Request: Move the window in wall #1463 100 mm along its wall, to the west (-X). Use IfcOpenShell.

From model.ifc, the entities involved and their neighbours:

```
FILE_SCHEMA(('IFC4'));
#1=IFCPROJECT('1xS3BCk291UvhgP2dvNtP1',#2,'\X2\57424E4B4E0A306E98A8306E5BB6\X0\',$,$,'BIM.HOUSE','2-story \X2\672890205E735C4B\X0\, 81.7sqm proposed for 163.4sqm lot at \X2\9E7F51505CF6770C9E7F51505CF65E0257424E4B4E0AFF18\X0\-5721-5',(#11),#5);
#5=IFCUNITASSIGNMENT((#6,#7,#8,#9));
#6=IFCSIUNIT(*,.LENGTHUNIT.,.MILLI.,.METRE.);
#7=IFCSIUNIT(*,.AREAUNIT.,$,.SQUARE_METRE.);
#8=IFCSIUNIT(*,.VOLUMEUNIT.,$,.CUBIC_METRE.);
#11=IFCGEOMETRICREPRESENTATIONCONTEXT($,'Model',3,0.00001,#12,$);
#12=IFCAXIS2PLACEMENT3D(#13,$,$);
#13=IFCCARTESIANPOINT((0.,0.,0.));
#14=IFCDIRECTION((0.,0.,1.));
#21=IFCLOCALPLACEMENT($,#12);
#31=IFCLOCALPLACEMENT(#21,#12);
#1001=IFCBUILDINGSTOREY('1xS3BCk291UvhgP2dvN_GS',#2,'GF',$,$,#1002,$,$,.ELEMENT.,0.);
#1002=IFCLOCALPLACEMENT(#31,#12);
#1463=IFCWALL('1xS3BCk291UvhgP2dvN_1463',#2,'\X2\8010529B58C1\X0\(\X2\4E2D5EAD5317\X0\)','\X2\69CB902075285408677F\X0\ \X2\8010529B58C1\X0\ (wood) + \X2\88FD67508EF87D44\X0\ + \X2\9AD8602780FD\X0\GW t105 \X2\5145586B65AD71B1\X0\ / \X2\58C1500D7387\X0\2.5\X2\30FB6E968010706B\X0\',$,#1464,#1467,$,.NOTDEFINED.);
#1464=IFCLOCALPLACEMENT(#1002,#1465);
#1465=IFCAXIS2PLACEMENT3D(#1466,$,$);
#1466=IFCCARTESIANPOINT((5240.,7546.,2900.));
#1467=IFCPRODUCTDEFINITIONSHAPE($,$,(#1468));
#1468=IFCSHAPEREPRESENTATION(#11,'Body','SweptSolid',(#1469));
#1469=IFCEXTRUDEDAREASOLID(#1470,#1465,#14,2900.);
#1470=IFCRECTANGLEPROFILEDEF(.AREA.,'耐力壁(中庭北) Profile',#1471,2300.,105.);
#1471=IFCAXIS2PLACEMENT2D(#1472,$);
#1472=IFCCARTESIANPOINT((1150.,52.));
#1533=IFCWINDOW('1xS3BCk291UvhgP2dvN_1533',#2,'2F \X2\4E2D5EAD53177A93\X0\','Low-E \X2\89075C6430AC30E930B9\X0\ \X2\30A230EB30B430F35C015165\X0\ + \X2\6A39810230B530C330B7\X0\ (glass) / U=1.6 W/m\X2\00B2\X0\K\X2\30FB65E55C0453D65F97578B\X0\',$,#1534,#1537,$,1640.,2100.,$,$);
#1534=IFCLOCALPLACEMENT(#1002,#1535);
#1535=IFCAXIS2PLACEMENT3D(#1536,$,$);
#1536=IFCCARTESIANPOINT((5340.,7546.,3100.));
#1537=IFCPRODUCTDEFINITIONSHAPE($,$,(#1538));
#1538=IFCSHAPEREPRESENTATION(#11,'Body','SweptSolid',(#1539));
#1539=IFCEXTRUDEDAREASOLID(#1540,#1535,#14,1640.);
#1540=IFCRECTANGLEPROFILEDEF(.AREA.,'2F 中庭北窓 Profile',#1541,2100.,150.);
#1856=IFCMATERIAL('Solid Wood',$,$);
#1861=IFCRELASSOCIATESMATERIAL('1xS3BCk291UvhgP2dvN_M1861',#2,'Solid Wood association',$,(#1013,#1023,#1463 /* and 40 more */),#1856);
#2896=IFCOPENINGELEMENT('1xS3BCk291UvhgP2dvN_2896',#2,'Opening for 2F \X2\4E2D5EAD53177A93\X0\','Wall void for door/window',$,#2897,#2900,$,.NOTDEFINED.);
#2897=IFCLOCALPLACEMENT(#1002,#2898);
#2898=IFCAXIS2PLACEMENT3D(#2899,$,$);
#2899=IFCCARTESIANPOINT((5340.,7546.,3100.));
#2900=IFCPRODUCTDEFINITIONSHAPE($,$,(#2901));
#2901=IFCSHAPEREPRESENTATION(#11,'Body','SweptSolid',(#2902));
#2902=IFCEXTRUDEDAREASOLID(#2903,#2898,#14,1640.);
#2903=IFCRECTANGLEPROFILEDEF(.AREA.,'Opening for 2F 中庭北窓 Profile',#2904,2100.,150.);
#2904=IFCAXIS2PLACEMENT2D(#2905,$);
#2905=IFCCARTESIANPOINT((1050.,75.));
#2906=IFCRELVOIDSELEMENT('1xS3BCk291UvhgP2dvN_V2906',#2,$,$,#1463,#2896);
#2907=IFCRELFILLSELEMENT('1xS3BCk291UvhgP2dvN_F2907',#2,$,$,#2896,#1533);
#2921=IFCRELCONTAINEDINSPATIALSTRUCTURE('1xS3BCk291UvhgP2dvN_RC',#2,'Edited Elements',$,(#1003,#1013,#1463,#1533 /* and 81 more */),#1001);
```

```python
import ifcopenshell
import ifcopenshell.api.geometry
import ifcopenshell.util.placement
import ifcopenshell.util.unit

model = ifcopenshell.open("model.ifc")
unit_scale = ifcopenshell.util.unit.calculate_unit_scale(model)

window = model.by_guid("1xS3BCk291UvhgP2dvN_1533")
opening = window.FillsVoids[0].RelatingOpeningElement
wall = opening.VoidsElements[0].RelatingBuildingElement

wall_matrix = ifcopenshell.util.placement.get_local_placement(wall.ObjectPlacement)
shift = wall_matrix[:3, 0] * -0.1 / unit_scale
before = ifcopenshell.util.placement.get_local_placement(window.ObjectPlacement)[:3, 3].copy()

# The window is not placed relative to its opening, so move both.
for product in (opening, window):
    matrix = ifcopenshell.util.placement.get_local_placement(product.ObjectPlacement)
    matrix[:3, 3] += shift
    ifcopenshell.api.geometry.edit_object_placement(model, product=product, matrix=matrix, is_si=False)

after = ifcopenshell.util.placement.get_local_placement(window.ObjectPlacement)[:3, 3]
print("window moved by", (after - before).round(3) + 0.0)

model.write("model-out.ifc")
```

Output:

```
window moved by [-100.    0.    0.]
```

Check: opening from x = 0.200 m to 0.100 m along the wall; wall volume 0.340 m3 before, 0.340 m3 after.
